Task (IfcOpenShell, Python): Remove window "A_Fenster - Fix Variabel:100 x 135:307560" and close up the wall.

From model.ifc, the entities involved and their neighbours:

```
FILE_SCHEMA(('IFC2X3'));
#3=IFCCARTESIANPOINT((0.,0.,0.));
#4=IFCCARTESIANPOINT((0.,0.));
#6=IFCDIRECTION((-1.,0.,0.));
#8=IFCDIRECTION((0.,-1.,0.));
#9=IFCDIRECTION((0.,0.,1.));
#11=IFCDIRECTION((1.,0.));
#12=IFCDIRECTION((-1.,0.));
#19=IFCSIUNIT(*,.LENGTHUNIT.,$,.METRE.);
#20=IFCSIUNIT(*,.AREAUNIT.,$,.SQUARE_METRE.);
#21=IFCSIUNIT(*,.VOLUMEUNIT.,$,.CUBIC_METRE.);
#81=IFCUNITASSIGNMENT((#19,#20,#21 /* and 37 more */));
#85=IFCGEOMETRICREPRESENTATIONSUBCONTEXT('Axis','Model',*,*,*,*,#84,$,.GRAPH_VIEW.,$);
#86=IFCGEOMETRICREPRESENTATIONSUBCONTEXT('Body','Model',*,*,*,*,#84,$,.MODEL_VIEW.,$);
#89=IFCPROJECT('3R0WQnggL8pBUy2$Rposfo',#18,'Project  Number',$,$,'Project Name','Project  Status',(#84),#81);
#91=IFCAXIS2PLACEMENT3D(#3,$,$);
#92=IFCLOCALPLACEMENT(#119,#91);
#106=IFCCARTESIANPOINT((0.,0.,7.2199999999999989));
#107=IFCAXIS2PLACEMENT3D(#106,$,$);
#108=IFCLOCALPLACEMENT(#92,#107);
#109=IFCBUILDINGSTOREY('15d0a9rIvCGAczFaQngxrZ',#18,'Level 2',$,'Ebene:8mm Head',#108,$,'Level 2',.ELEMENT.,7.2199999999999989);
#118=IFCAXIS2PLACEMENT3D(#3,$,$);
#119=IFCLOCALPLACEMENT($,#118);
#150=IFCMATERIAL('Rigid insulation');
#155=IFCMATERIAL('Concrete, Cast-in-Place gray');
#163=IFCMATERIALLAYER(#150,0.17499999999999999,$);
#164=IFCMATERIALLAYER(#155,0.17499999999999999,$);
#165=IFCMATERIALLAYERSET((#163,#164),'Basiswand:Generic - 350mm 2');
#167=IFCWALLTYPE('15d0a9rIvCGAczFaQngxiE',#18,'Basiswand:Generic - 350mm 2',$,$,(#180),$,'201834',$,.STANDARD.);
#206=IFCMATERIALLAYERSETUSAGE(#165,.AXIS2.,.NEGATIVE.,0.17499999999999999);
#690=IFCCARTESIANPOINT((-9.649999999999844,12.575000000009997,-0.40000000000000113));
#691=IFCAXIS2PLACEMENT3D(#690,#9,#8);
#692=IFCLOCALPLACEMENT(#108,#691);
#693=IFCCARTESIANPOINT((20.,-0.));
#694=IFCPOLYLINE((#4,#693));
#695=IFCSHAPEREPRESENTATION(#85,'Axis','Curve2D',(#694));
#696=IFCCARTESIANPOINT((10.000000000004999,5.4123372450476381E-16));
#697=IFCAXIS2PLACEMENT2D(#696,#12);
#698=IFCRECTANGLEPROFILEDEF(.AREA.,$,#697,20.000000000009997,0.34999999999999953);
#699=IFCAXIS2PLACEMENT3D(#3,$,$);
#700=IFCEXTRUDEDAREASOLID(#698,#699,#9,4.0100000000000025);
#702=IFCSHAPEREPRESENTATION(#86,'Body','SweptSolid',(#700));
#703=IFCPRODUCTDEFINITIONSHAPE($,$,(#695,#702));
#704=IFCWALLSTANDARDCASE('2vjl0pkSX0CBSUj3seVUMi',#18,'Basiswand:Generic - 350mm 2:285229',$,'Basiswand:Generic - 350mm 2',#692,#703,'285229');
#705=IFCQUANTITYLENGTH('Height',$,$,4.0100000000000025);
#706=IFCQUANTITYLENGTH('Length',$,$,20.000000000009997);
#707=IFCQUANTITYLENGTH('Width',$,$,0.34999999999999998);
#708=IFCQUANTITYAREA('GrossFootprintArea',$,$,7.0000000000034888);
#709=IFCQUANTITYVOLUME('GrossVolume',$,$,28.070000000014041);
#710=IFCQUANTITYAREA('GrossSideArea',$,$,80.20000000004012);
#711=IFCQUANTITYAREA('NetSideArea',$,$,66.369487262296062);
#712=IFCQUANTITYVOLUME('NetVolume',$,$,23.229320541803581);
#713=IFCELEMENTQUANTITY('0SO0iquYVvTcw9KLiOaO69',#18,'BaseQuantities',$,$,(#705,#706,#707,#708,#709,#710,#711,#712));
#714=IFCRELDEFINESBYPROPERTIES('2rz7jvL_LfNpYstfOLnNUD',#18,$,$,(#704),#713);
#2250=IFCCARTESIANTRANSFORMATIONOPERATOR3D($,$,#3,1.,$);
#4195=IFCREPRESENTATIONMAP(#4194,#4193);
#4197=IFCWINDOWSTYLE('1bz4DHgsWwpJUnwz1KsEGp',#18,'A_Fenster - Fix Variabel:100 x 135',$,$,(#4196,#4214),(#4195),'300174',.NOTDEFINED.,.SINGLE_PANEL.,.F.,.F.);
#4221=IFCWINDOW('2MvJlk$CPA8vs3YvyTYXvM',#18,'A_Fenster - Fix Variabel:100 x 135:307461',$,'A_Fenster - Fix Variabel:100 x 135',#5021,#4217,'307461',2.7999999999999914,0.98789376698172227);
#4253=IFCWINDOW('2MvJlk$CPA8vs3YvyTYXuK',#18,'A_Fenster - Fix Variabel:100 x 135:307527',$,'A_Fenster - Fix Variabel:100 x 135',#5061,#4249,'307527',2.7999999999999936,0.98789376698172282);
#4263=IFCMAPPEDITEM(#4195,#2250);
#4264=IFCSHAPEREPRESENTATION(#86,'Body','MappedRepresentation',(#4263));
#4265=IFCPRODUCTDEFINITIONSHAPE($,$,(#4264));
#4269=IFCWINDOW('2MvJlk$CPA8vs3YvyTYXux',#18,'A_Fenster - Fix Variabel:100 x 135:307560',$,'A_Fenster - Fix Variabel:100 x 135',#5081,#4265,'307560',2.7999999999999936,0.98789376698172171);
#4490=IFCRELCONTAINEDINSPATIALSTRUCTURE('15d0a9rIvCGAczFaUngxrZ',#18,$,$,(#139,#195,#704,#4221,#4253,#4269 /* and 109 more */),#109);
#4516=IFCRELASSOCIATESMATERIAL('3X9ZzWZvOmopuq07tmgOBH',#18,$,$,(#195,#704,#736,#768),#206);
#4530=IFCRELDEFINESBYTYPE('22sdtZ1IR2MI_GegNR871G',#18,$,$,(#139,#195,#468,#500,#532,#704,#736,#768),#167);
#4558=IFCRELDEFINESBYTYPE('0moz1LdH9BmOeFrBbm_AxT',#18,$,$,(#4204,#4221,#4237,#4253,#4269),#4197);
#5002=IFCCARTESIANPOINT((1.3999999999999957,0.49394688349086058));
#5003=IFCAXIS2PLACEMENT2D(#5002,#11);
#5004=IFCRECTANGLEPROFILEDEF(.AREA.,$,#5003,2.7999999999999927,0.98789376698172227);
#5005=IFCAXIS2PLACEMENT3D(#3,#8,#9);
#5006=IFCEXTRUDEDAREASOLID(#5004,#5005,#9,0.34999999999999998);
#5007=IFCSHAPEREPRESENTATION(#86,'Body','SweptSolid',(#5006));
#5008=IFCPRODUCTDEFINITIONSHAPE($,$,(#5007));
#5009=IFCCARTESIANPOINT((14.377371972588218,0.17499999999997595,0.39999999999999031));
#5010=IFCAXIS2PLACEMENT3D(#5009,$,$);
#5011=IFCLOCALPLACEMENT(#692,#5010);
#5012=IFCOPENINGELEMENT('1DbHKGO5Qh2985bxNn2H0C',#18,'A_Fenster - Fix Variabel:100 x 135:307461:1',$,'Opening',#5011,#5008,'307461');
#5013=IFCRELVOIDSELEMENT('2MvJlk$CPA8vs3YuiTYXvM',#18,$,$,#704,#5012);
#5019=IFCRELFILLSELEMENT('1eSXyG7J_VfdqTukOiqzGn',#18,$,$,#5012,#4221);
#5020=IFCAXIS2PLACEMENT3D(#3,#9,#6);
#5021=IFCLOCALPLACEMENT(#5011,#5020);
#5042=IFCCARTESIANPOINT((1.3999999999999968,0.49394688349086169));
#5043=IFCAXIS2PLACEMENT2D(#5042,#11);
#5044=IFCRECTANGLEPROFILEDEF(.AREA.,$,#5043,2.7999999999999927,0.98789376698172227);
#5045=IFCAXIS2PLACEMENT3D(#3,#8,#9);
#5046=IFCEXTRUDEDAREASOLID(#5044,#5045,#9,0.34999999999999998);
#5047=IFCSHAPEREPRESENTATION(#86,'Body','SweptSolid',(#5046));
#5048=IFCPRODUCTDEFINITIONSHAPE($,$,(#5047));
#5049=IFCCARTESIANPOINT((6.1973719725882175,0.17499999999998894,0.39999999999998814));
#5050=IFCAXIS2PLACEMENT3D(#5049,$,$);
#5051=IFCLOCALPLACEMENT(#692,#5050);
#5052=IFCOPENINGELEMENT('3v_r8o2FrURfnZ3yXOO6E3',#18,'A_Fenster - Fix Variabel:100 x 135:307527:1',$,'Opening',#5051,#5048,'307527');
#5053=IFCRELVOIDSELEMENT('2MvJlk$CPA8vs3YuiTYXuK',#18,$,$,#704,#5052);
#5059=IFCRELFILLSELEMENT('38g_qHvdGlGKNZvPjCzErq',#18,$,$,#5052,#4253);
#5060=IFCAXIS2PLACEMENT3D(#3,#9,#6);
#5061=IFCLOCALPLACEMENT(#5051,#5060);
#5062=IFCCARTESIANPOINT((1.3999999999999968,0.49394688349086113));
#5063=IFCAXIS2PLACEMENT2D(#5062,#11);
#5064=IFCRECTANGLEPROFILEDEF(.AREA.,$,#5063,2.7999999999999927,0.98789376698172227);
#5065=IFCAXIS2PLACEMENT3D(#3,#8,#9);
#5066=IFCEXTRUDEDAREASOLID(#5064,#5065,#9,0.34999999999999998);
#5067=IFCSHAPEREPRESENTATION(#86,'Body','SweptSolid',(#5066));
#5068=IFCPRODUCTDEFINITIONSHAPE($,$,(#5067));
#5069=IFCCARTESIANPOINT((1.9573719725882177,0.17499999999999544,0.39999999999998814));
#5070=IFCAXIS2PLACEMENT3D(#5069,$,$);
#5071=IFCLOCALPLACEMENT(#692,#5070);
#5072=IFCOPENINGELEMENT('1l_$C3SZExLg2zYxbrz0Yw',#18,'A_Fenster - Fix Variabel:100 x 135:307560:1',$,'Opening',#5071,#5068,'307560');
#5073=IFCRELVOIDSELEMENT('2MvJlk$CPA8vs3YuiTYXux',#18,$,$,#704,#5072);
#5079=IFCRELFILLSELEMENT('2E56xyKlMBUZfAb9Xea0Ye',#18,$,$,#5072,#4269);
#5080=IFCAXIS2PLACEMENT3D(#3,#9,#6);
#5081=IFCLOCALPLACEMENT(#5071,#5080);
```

```python
import ifcopenshell
import ifcopenshell.api.feature
import ifcopenshell.api.pset
import ifcopenshell.api.root
import ifcopenshell.geom
import ifcopenshell.util.element
import ifcopenshell.util.shape
import ifcopenshell.util.unit

model = ifcopenshell.open("model.ifc")
area_scale = ifcopenshell.util.unit.calculate_unit_scale(model, "AREAUNIT")
volume_scale = ifcopenshell.util.unit.calculate_unit_scale(model, "VOLUMEUNIT")
settings = ifcopenshell.geom.settings()


def volume(element):
    """Net volume in cubic metres, openings subtracted."""
    shape = ifcopenshell.geom.create_shape(settings, element)
    return ifcopenshell.util.shape.get_volume(shape.geometry)


window = model.by_id(4269)
opening = window.FillsVoids[0].RelatingOpeningElement
wall = opening.VoidsElements[0].RelatingBuildingElement
before = volume(wall)

ifcopenshell.api.root.remove_product(model, product=window)
ifcopenshell.api.feature.remove_feature(model, feature=opening)

after = volume(wall)
thickness = 0.35  # wall thickness in metres

# Update the wall's stored quantities.
qto = model.by_id(ifcopenshell.util.element.get_pset(wall, "BaseQuantities", should_inherit=False)["id"])
ifcopenshell.api.pset.edit_qto(model, qto=qto, properties={
    "NetSideArea": after / thickness / area_scale,
    "NetVolume": after / volume_scale,
})

print(f"wall volume {before:.3f} -> {after:.3f} m3")

model.write("model_updated.ifc")
```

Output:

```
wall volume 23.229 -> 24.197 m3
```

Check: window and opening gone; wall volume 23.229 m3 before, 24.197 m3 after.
